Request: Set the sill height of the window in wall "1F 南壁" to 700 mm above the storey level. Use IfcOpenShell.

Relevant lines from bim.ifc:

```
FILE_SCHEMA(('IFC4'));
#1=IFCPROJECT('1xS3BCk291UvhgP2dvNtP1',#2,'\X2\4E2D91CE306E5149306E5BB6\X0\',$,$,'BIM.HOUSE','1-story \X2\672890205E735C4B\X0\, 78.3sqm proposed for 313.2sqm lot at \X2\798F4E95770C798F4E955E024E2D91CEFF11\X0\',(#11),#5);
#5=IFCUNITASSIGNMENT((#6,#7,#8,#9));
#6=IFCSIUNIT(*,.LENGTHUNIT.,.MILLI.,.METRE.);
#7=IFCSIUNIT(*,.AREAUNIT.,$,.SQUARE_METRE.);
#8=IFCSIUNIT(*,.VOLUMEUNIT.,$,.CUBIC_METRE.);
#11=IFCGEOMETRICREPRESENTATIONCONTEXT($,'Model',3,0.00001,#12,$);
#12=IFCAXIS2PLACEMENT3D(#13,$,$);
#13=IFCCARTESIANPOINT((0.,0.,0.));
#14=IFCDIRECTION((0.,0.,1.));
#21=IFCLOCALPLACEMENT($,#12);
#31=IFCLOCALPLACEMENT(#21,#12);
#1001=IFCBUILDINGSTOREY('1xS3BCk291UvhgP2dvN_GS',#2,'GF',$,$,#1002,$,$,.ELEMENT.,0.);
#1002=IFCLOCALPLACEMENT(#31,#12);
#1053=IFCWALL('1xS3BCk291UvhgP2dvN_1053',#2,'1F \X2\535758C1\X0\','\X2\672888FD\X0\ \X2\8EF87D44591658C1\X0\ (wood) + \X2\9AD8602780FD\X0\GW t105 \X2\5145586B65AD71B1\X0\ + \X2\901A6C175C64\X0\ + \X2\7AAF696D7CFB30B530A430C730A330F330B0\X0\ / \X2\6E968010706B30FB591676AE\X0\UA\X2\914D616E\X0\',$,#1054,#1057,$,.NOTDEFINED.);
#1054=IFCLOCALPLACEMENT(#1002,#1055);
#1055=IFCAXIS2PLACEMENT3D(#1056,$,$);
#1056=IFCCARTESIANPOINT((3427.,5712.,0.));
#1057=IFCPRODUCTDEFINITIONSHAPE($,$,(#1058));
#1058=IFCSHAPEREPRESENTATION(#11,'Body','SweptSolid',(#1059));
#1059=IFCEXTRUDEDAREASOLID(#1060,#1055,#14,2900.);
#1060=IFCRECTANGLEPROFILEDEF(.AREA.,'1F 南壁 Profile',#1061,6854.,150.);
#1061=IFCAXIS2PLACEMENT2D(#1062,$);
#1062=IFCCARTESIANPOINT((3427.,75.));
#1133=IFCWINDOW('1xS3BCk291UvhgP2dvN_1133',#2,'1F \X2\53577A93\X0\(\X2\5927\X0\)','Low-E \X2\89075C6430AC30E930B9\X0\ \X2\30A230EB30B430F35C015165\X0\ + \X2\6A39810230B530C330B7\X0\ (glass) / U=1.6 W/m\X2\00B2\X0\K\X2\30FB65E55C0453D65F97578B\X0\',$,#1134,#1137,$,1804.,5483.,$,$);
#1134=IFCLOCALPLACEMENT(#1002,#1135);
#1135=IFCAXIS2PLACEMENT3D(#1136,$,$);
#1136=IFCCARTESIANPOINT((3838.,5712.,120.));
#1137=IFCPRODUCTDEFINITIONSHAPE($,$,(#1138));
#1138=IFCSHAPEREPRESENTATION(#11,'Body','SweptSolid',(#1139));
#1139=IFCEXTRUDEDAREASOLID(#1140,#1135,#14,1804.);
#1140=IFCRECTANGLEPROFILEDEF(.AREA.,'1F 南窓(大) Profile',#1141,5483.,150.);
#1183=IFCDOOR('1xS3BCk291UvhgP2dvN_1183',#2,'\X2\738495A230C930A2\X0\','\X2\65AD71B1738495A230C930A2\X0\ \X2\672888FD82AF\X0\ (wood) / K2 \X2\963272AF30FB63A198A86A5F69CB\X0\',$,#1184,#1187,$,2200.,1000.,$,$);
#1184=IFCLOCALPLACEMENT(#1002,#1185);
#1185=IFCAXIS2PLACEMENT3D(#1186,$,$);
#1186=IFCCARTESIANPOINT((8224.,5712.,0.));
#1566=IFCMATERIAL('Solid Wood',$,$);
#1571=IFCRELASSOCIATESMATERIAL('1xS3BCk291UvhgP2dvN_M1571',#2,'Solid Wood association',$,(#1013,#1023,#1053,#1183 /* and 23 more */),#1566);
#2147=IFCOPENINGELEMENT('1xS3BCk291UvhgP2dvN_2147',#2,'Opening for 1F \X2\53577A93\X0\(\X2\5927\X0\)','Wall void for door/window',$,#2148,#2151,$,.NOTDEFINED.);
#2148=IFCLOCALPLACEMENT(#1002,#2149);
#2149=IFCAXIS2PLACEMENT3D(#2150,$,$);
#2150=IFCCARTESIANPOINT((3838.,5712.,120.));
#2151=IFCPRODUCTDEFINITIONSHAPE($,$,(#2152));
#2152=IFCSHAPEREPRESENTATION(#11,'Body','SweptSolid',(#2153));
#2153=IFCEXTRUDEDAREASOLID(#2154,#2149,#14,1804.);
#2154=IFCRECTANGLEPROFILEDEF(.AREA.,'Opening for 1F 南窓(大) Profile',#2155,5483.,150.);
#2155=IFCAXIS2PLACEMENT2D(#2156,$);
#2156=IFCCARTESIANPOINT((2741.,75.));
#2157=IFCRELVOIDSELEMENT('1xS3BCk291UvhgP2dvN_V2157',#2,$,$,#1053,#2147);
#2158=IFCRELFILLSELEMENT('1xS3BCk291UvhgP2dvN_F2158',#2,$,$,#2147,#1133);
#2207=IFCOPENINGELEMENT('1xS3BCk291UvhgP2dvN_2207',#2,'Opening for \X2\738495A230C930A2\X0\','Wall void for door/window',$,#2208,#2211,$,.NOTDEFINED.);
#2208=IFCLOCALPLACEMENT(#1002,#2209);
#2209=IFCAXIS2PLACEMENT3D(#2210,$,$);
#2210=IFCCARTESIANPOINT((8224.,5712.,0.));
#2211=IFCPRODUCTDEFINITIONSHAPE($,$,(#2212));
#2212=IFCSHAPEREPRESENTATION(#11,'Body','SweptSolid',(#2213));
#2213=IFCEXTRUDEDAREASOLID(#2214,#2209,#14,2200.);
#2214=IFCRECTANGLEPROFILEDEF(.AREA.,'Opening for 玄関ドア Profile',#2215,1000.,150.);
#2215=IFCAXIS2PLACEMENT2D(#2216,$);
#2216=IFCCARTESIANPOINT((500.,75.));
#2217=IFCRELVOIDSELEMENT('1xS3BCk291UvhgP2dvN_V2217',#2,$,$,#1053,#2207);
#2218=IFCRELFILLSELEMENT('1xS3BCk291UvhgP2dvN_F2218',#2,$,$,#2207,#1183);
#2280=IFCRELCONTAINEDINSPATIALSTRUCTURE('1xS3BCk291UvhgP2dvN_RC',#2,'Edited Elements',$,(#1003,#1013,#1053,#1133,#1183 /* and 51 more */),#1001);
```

```python
import numpy as np
import ifcopenshell
import ifcopenshell.api.geometry
import ifcopenshell.geom
import ifcopenshell.util.element
import ifcopenshell.util.placement
import ifcopenshell.util.shape
import ifcopenshell.util.unit

model = ifcopenshell.open("bim.ifc")
unit_scale = ifcopenshell.util.unit.calculate_unit_scale(model)

window = model.by_guid("1xS3BCk291UvhgP2dvN_1133")
opening = window.FillsVoids[0].RelatingOpeningElement
storey = ifcopenshell.util.element.get_container(window, ifc_class="IfcBuildingStorey")
level = ifcopenshell.util.placement.get_local_placement(storey.ObjectPlacement)[2, 3]

# The opening's origin need not be at the sill, so measure its lowest point.
shape = ifcopenshell.geom.create_shape(ifcopenshell.geom.settings(), opening)
bottom = ifcopenshell.util.shape.get_shape_bottom_elevation(shape, shape.geometry) / unit_scale
dz = level + 0.7 / unit_scale - bottom

shift = np.array([0.0, 0.0, dz])
# The window is not placed relative to its opening, so move both.
for product in (opening, window):
    matrix = ifcopenshell.util.placement.get_local_placement(product.ObjectPlacement)
    matrix[:3, 3] += shift
    ifcopenshell.api.geometry.edit_object_placement(model, product=product, matrix=matrix, is_si=False)

print(f"moved by {dz * unit_scale:+.3f} m")

model.write("bim_edited.ifc")
```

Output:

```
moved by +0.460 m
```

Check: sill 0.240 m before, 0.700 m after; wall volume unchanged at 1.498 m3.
